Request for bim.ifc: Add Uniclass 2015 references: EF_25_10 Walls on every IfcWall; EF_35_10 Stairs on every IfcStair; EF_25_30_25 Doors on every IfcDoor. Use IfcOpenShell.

First a look at what the model holds.

```python
import ifcopenshell

model = ifcopenshell.open("bim.ifc")
print(model.schema)
print("classifications:", [c.Name for c in model.by_type("IfcClassification")])
for ifc_class in ("IfcDoor", "IfcRoof", "IfcStair", "IfcWall", "IfcWindow"):
    print(ifc_class, len(model.by_type(ifc_class)))
```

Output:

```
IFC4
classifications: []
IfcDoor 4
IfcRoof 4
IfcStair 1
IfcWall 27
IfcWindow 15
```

```python
import ifcopenshell
import ifcopenshell.api.classification

model = ifcopenshell.open("bim.ifc")

system = ifcopenshell.api.classification.add_classification(model, classification="Uniclass 2015")

codes = {
    "IfcWall": ("EF_25_10", "Walls"),
    "IfcStair": ("EF_35_10", "Stairs"),
    "IfcDoor": ("EF_25_30_25", "Doors"),
}
for ifc_class, (code, name) in codes.items():
    products = model.by_type(ifc_class)
    ifcopenshell.api.classification.add_reference(
        model, products=products, classification=system, identification=code, name=name
    )
    print(code, len(products))

model.write("bim-out.ifc")
```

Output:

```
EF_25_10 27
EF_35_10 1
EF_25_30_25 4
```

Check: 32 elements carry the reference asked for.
